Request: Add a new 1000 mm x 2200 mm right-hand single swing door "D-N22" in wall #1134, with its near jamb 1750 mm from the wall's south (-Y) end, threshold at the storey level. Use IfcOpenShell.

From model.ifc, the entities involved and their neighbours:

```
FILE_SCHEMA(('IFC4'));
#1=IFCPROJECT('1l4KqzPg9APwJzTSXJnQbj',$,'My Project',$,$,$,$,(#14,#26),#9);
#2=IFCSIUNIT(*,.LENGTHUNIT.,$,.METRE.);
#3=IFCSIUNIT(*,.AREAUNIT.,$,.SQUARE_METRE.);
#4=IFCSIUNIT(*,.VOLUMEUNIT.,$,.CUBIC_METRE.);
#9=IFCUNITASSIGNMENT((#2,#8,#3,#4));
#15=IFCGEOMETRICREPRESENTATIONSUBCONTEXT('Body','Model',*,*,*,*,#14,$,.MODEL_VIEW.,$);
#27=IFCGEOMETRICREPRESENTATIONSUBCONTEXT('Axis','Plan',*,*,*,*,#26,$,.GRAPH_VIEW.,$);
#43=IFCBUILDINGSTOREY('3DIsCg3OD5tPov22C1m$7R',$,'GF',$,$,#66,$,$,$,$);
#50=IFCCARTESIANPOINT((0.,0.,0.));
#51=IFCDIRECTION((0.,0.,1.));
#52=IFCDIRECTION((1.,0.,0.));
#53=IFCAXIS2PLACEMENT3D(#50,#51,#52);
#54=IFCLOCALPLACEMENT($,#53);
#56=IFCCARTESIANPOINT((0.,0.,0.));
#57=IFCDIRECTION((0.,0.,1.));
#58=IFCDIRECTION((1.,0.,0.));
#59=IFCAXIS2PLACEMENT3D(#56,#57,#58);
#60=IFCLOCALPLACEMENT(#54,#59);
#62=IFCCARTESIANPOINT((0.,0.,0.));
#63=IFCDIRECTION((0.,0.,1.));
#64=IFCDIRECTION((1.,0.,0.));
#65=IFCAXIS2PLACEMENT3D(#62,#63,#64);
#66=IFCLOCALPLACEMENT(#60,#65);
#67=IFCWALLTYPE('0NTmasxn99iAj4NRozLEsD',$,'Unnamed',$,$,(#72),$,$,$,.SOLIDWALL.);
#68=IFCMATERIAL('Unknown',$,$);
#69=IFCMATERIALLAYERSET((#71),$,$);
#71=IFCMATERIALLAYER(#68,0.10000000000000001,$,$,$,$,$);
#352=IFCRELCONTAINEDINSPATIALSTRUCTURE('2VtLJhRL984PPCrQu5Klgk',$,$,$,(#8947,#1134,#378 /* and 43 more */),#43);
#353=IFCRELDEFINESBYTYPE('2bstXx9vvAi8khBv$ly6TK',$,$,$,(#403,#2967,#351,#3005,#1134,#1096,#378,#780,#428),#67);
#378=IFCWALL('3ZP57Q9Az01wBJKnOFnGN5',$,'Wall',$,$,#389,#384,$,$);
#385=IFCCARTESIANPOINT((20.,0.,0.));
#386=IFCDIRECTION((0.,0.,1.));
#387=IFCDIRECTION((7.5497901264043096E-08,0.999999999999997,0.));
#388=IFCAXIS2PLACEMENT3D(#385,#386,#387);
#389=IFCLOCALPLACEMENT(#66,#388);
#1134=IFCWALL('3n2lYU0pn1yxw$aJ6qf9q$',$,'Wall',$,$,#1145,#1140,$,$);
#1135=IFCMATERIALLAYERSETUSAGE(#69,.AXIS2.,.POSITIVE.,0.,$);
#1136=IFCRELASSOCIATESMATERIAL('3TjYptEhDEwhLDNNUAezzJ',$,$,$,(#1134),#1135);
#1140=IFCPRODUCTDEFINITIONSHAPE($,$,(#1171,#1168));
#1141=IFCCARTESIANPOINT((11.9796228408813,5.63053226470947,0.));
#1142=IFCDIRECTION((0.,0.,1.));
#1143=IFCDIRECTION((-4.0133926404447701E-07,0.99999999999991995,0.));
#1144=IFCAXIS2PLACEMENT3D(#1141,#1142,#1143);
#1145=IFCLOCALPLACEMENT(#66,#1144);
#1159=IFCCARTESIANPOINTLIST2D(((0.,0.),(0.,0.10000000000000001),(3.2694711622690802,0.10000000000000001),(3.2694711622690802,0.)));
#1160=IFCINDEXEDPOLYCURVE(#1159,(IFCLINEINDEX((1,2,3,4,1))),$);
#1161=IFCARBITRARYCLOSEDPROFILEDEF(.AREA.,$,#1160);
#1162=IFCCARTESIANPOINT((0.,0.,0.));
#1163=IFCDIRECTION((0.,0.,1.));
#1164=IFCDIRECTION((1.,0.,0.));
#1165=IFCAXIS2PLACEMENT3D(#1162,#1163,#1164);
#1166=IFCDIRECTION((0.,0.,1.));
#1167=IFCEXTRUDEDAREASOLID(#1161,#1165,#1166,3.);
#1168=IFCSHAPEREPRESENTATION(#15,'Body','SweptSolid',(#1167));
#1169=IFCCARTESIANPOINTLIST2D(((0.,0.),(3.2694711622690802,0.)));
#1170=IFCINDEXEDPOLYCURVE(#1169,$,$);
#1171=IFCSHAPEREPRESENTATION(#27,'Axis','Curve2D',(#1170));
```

```python
import numpy as np
import ifcopenshell
import ifcopenshell.api.feature
import ifcopenshell.api.geometry
import ifcopenshell.api.root
import ifcopenshell.api.spatial
import ifcopenshell.geom
import ifcopenshell.util.element
import ifcopenshell.util.placement
import ifcopenshell.util.representation
import ifcopenshell.util.shape
import ifcopenshell.util.unit

model = ifcopenshell.open("model.ifc")
unit_scale = ifcopenshell.util.unit.calculate_unit_scale(model)
settings = ifcopenshell.geom.settings()


def volume(element):
    """Net volume in cubic metres, openings subtracted."""
    shape = ifcopenshell.geom.create_shape(settings, element)
    return ifcopenshell.util.shape.get_volume(shape.geometry)


wall = model.by_guid("3n2lYU0pn1yxw$aJ6qf9q$")
storey = ifcopenshell.util.element.get_container(wall, ifc_class="IfcBuildingStorey")
context = ifcopenshell.util.representation.get_context(model, "Model", "Body", "MODEL_VIEW")
before = volume(wall)

width, height, from_end, sill = 1, 2.2, 1.75, 0.0  # metres

# The wall runs along its own X axis, and the end named is its -X end.
wall_shape = ifcopenshell.geom.create_shape(settings, wall)
x, y, z = ifcopenshell.util.shape.get_vertices(wall_shape.geometry).T
start = x.min() + from_end
face, thickness = float(y.min()), float(y.max() - y.min())
wall_matrix = ifcopenshell.util.placement.get_local_placement(wall.ObjectPlacement)
level = ifcopenshell.util.placement.get_local_placement(storey.ObjectPlacement)[2, 3]


def in_wall(x, y):
    """Placement at x, y metres in the wall's axes, at sill height."""
    matrix = wall_matrix.copy()
    matrix[:, 3] = wall_matrix @ np.array([x / unit_scale, y / unit_scale, 0.0, 1.0])
    matrix[2, 3] = level + sill / unit_scale
    return matrix


# Opening: a box that overshoots both wall faces by 50 mm.
opening = ifcopenshell.api.root.create_entity(model, ifc_class="IfcOpeningElement", predefined_type="OPENING")
box = ifcopenshell.api.geometry.add_wall_representation(
    model, context=context, length=width, height=height, thickness=thickness + 0.1
)
ifcopenshell.api.geometry.assign_representation(model, product=opening, representation=box)
ifcopenshell.api.geometry.edit_object_placement(model, product=opening, matrix=in_wall(start, face - 0.05), is_si=False)
ifcopenshell.api.feature.add_feature(model, feature=opening, element=wall)

door = ifcopenshell.api.root.create_entity(model, ifc_class="IfcDoor", name="D-N22", predefined_type="DOOR")
door.OverallWidth, door.OverallHeight = width / unit_scale, height / unit_scale
door.OperationType = "SINGLE_SWING_RIGHT"
body = ifcopenshell.api.geometry.add_door_representation(
    model,
    context=context,
    overall_width=door.OverallWidth,
    overall_height=door.OverallHeight,
    operation_type="SINGLE_SWING_RIGHT",
    lining_properties={"LiningDepth": thickness / unit_scale, "ThresholdDepth": thickness / unit_scale},
)
ifcopenshell.api.geometry.assign_representation(model, product=door, representation=body)
ifcopenshell.api.spatial.assign_container(model, products=[door], relating_structure=storey)
ifcopenshell.api.feature.add_filling(model, opening=opening, element=door)

# The lining spans the wall, so the door starts at the wall face.
ifcopenshell.api.geometry.edit_object_placement(model, product=door, matrix=in_wall(start, face), is_si=False)

after = volume(wall)

print(f"wall volume {before:.3f} -> {after:.3f} m3")

model.write("model_v2.ifc")
```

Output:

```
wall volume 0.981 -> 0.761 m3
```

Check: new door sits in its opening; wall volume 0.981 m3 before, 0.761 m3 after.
